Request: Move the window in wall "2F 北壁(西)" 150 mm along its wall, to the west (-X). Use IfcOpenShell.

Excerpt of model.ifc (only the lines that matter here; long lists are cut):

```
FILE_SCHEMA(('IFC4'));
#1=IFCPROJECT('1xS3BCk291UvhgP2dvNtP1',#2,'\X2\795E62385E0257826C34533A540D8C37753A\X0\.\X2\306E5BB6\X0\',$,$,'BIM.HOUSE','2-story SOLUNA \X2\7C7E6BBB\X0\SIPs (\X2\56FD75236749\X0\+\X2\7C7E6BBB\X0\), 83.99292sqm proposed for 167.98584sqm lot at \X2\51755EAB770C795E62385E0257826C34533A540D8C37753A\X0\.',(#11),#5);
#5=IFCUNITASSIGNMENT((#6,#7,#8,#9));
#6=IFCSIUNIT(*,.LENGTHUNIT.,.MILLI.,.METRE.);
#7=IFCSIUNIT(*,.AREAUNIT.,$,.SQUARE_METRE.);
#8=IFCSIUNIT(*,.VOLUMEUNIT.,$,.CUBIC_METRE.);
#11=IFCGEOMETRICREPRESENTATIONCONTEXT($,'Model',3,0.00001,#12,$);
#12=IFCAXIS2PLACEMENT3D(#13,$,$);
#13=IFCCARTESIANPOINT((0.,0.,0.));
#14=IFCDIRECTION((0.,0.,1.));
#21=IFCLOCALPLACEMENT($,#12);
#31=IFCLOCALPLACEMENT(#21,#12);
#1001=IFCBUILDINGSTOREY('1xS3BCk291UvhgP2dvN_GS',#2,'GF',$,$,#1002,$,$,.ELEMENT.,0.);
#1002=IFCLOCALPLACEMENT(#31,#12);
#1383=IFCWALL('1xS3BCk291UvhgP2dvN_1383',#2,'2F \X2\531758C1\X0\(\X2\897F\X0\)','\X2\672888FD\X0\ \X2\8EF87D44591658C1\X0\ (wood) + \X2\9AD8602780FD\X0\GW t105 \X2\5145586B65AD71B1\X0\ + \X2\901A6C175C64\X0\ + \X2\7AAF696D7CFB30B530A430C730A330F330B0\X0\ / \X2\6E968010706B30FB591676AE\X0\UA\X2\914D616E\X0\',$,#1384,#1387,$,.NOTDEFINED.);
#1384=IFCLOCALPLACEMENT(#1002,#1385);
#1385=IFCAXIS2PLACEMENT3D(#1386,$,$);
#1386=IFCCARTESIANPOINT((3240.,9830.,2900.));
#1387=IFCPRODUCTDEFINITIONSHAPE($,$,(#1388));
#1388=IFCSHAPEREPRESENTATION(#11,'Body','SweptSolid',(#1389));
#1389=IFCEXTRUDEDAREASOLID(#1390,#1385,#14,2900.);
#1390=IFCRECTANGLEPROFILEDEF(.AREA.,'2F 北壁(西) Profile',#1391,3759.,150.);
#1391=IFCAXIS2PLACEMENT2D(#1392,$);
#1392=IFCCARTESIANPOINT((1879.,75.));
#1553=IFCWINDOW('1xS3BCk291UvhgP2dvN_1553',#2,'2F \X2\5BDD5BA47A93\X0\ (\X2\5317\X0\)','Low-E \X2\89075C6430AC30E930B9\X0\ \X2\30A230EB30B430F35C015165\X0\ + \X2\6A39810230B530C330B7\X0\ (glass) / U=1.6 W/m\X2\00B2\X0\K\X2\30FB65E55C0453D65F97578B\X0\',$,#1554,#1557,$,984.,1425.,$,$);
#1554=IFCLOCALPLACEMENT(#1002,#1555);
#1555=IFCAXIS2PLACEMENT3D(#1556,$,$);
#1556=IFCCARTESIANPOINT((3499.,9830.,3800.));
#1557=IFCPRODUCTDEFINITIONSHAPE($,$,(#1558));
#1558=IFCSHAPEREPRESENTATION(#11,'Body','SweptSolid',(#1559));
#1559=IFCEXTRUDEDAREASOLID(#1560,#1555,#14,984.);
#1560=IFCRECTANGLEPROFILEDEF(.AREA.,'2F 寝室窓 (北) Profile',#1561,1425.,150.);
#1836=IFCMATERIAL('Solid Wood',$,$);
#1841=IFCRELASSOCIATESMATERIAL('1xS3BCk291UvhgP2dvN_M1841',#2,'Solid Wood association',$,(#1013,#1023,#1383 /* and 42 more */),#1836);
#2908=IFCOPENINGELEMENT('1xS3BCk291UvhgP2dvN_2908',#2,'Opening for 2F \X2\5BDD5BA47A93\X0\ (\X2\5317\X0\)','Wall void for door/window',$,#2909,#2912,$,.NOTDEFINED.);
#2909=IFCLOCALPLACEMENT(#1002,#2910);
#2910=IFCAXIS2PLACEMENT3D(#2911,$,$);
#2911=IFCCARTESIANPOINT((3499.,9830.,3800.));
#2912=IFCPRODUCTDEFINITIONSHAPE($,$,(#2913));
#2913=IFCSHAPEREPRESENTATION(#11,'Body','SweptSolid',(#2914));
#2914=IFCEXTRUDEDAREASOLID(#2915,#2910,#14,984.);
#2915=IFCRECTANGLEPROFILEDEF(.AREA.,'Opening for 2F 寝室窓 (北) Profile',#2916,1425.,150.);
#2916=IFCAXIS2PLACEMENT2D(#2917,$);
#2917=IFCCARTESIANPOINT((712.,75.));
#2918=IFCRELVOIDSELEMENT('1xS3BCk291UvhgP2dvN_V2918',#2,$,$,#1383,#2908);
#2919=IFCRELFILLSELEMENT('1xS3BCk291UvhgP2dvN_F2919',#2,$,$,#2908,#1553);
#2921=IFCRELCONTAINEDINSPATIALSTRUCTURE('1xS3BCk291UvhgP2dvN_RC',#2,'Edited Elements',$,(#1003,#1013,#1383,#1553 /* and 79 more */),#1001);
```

```python
import ifcopenshell
import ifcopenshell.api.geometry
import ifcopenshell.util.placement
import ifcopenshell.util.unit

model = ifcopenshell.open("model.ifc")
unit_scale = ifcopenshell.util.unit.calculate_unit_scale(model)

window = model.by_guid("1xS3BCk291UvhgP2dvN_1553")
opening = window.FillsVoids[0].RelatingOpeningElement
wall = opening.VoidsElements[0].RelatingBuildingElement

wall_matrix = ifcopenshell.util.placement.get_local_placement(wall.ObjectPlacement)
shift = wall_matrix[:3, 0] * -0.15 / unit_scale
before = ifcopenshell.util.placement.get_local_placement(window.ObjectPlacement)[:3, 3].copy()

# The window is not placed relative to its opening, so move both.
for product in (opening, window):
    matrix = ifcopenshell.util.placement.get_local_placement(product.ObjectPlacement)
    matrix[:3, 3] += shift
    ifcopenshell.api.geometry.edit_object_placement(model, product=product, matrix=matrix, is_si=False)

after = ifcopenshell.util.placement.get_local_placement(window.ObjectPlacement)[:3, 3]
print("window moved by", (after - before).round(3) + 0.0)

model.write("model_edited.ifc")
```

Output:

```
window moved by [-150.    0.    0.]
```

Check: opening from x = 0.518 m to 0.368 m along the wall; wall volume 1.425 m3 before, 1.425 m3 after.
